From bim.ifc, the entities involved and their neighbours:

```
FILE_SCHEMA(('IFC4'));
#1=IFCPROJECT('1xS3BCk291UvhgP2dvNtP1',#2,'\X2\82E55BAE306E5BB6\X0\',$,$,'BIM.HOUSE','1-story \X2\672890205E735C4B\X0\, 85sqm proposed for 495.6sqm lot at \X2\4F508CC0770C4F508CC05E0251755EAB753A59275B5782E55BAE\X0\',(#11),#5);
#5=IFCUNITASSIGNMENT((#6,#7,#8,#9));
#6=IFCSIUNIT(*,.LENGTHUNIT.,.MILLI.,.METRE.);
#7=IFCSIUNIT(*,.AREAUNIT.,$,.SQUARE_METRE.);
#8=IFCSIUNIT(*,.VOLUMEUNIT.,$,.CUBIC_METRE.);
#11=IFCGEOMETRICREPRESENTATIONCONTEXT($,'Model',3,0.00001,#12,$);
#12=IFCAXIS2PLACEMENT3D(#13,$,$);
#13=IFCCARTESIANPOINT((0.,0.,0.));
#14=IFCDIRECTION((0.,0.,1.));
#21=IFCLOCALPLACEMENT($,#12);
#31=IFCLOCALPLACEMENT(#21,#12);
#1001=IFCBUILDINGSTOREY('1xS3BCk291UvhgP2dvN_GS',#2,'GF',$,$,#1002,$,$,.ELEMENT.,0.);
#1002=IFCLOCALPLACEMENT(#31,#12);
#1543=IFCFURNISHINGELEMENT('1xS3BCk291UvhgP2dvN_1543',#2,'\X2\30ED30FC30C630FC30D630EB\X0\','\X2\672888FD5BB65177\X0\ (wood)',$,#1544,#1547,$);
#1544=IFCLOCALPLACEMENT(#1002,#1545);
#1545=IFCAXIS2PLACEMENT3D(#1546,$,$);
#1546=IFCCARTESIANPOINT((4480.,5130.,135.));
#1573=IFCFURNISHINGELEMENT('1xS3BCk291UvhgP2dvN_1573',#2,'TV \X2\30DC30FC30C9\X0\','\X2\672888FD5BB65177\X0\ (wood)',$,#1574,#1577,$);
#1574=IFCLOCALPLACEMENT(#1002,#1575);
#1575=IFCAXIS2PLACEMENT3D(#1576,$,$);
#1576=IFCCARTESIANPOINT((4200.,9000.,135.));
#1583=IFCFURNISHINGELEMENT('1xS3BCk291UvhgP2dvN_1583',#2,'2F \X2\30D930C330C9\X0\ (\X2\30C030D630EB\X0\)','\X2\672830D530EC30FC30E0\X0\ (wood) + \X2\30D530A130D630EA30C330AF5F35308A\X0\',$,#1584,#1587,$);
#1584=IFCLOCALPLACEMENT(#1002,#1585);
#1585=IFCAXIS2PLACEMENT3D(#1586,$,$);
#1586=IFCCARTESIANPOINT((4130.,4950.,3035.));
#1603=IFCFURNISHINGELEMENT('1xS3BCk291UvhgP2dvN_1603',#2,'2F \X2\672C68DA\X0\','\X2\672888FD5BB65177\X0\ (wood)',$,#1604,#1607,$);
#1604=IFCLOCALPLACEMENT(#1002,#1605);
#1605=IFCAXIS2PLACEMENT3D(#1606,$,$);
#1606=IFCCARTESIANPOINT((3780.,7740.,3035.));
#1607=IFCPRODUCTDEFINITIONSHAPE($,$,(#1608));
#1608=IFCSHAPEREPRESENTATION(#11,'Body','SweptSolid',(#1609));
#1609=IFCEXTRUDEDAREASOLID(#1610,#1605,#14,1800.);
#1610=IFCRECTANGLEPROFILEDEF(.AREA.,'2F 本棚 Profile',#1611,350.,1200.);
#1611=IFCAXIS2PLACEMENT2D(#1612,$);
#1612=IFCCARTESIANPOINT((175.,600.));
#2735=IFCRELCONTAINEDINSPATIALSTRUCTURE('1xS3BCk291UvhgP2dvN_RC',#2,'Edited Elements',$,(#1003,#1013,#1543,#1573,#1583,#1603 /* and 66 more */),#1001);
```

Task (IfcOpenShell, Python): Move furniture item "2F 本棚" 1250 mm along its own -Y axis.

```python
import ifcopenshell
import ifcopenshell.api.geometry
import ifcopenshell.util.placement
import ifcopenshell.util.unit

model = ifcopenshell.open("bim.ifc")
unit_scale = ifcopenshell.util.unit.calculate_unit_scale(model)

item = model.by_guid("1xS3BCk291UvhgP2dvN_1603")
matrix = ifcopenshell.util.placement.get_local_placement(item.ObjectPlacement)
matrix[:3, 3] -= matrix[:3, 1] * 1.25 / unit_scale
ifcopenshell.api.geometry.edit_object_placement(model, product=item, matrix=matrix, is_si=False)

print(ifcopenshell.util.placement.get_local_placement(item.ObjectPlacement).round(3) + 0.0)

model.write("bim-out.ifc")
```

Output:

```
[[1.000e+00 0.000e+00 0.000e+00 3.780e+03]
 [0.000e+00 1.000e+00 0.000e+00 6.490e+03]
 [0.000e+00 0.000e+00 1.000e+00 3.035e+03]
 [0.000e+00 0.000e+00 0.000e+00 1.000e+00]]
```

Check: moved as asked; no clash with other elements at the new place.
